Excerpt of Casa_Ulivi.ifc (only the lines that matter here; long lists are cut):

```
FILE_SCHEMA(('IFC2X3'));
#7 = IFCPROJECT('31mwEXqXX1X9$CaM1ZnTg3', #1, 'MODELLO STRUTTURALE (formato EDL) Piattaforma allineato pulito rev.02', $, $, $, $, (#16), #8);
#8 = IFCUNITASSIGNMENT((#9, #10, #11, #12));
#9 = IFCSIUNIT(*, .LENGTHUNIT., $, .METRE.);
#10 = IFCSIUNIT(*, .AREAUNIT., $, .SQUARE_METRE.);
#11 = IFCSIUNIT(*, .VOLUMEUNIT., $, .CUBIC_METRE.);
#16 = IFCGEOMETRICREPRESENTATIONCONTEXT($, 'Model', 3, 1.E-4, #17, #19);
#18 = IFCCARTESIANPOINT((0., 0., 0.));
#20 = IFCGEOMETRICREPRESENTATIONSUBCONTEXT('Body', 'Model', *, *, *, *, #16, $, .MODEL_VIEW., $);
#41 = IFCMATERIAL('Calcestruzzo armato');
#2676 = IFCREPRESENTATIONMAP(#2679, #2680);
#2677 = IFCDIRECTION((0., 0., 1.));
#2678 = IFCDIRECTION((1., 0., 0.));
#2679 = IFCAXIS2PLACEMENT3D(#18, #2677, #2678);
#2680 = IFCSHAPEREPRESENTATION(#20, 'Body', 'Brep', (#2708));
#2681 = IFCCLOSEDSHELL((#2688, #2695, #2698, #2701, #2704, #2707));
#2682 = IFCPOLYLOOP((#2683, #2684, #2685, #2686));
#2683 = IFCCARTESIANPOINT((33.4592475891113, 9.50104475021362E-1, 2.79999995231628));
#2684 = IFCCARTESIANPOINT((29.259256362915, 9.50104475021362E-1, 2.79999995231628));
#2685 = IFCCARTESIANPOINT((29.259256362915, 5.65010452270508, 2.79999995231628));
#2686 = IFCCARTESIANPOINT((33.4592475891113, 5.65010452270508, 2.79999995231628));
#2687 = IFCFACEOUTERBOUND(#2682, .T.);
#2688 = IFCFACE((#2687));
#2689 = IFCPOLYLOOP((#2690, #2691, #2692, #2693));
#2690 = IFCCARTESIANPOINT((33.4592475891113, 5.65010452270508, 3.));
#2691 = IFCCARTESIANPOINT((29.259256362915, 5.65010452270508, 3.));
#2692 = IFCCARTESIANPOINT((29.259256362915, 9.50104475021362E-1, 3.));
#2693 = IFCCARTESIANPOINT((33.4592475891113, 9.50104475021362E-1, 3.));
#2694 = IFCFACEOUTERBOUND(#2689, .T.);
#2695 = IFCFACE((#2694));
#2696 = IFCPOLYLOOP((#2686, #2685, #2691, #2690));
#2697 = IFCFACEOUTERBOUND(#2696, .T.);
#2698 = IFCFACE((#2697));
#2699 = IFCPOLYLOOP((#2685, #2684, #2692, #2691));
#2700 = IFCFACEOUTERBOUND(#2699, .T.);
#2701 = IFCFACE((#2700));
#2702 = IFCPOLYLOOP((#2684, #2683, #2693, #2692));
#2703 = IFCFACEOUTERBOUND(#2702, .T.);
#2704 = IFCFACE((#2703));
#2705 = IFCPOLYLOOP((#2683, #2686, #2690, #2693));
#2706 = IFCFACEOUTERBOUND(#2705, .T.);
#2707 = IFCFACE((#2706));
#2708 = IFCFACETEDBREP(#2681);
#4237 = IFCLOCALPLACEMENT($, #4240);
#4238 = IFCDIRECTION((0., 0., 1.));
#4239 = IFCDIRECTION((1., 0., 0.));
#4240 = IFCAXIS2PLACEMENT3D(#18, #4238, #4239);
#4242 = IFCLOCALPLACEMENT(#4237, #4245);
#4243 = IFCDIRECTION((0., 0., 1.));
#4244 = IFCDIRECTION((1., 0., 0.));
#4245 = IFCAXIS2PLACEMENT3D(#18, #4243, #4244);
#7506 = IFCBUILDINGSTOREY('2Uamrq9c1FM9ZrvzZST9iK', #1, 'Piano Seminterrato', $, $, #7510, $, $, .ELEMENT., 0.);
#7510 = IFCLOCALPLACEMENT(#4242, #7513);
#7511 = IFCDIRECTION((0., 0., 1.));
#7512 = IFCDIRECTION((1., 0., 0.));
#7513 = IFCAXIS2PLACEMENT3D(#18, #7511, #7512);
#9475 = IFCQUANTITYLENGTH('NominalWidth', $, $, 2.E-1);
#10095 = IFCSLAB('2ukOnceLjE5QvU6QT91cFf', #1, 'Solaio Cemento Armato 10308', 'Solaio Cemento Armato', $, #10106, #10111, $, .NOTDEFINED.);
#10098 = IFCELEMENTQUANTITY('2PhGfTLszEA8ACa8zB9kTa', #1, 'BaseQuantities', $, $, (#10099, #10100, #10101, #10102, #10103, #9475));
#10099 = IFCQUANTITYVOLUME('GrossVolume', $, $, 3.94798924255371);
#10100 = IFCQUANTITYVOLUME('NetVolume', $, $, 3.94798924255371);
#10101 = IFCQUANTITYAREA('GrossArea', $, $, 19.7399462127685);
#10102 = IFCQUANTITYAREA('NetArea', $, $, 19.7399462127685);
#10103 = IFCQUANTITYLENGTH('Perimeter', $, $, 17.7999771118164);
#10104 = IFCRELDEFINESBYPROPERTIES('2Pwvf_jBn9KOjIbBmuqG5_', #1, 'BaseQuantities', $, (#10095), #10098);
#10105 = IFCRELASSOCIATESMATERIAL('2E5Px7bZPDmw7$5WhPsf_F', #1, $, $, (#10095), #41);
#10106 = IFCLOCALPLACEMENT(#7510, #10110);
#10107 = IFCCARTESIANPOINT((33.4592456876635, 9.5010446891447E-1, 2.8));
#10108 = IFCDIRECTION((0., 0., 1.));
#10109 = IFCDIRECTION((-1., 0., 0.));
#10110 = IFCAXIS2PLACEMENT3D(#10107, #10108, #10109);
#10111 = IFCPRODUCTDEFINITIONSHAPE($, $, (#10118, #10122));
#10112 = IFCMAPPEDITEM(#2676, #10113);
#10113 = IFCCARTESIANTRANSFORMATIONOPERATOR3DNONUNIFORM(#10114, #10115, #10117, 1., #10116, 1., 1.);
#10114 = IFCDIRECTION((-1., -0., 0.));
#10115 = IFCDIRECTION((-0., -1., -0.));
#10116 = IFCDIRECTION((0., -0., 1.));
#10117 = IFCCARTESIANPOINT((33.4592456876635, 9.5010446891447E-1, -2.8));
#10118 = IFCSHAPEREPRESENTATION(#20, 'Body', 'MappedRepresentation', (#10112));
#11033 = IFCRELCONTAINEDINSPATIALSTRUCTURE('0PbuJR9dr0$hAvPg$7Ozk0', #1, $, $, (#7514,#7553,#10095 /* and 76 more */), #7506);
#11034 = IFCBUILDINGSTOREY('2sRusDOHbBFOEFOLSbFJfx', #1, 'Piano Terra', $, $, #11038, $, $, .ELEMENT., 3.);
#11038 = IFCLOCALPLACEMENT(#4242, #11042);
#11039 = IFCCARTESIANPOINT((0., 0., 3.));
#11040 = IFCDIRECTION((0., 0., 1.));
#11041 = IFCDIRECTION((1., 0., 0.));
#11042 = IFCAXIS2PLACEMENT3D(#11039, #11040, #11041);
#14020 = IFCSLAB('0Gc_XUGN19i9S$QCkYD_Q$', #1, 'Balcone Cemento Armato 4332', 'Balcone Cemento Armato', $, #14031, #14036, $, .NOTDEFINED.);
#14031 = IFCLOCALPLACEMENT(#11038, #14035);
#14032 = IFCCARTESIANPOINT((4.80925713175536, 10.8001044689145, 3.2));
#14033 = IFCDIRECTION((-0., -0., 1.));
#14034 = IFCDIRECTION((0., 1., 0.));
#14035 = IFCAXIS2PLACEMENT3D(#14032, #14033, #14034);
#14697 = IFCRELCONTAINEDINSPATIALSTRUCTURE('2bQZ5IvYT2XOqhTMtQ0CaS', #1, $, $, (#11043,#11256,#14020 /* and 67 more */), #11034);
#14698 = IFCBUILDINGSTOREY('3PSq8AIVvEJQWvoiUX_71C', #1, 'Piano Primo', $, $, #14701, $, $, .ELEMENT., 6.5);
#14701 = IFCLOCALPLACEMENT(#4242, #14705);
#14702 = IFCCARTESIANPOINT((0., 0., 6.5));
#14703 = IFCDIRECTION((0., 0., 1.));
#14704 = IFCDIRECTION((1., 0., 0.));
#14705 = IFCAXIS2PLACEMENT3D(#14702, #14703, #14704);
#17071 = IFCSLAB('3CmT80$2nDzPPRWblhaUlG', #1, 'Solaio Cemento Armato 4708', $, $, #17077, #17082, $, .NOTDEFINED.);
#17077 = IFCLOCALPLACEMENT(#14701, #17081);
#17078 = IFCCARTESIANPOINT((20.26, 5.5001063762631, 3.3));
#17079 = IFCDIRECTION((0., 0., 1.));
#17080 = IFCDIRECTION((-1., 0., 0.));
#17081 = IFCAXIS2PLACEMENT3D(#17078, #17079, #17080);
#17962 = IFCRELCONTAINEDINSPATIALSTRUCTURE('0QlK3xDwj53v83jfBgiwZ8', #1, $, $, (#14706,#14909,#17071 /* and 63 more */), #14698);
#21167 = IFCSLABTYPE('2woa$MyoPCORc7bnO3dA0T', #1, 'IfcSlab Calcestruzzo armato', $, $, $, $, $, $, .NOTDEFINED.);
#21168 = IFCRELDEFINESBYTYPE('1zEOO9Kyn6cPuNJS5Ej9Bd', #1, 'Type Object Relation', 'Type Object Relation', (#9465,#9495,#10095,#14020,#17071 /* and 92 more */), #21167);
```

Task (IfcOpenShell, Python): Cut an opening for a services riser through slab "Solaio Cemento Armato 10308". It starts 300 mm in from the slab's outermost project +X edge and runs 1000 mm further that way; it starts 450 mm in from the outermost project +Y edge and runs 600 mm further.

```python
import numpy as np
import ifcopenshell
import ifcopenshell.api.feature
import ifcopenshell.api.geometry
import ifcopenshell.api.pset
import ifcopenshell.api.root
import ifcopenshell.geom
import ifcopenshell.util.element
import ifcopenshell.util.placement
import ifcopenshell.util.representation
import ifcopenshell.util.shape
import ifcopenshell.util.unit

model = ifcopenshell.open("Casa_Ulivi.ifc")
unit_scale = ifcopenshell.util.unit.calculate_unit_scale(model)
area_scale = ifcopenshell.util.unit.calculate_unit_scale(model, "AREAUNIT")
volume_scale = ifcopenshell.util.unit.calculate_unit_scale(model, "VOLUMEUNIT")
settings = ifcopenshell.geom.settings()


def volume(element):
    """Net volume in cubic metres, openings subtracted."""
    shape = ifcopenshell.geom.create_shape(settings, element)
    return ifcopenshell.util.shape.get_volume(shape.geometry)


slab = model.by_id(10095)
before = volume(slab)

# Extent in the slab's own axes, in metres. The edges named are its -X and -Y sides.
slab_shape = ifcopenshell.geom.create_shape(settings, slab)
vertices = ifcopenshell.util.shape.get_vertices(slab_shape.geometry)
x_min, y_min, bottom = vertices.min(axis=0)
top = vertices[:, 2].max()

opening = ifcopenshell.api.root.create_entity(model, ifc_class="IfcOpeningElement", name="Services riser opening")
context = ifcopenshell.util.representation.get_context(model, "Model", "Body", "MODEL_VIEW")
width, depth = 1, 0.6
outline = [(0.0, 0.0), (width, 0.0), (width, depth), (0.0, depth), (0.0, 0.0)]
# Overshoot both faces by 50 mm so the cut is clean.
shape = ifcopenshell.api.geometry.add_slab_representation(
    model, context=context, depth=top - bottom + 0.1, polyline=outline
)
ifcopenshell.api.geometry.assign_representation(model, product=opening, representation=shape)

matrix = ifcopenshell.util.placement.get_local_placement(slab.ObjectPlacement)
matrix[:, 3] = matrix @ np.append(np.array([x_min + 0.3, y_min + 0.45, bottom - 0.05]) / unit_scale, 1.0)
ifcopenshell.api.geometry.edit_object_placement(model, product=opening, matrix=matrix, is_si=False)
ifcopenshell.api.feature.add_feature(model, feature=opening, element=slab)

after = volume(slab)

# Update the slab's stored quantities.
qto = model.by_id(ifcopenshell.util.element.get_pset(slab, "BaseQuantities", should_inherit=False)["id"])
ifcopenshell.api.pset.edit_qto(model, qto=qto, properties={
    "NetVolume": after / volume_scale,
    "NetArea": after / (top - bottom) / area_scale,
})

print(f"slab volume {before:.3f} -> {after:.3f} m3")

model.write("Casa_Ulivi_edited.ifc")
```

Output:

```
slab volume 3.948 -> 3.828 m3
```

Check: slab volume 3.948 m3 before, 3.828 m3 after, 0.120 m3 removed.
